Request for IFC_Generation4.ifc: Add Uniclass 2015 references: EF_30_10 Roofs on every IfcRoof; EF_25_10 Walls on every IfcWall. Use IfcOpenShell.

First a look at what the model holds.

```python
import ifcopenshell

model = ifcopenshell.open("IFC_Generation4.ifc")
print(model.schema)
print("classifications:", [c.Name for c in model.by_type("IfcClassification")])
for ifc_class in ("IfcDoor", "IfcRoof", "IfcStair", "IfcWall", "IfcWindow"):
    print(ifc_class, len(model.by_type(ifc_class)))
```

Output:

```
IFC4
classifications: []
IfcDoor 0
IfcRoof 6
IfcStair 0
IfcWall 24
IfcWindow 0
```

```python
import ifcopenshell
import ifcopenshell.api.classification

model = ifcopenshell.open("IFC_Generation4.ifc")

system = ifcopenshell.api.classification.add_classification(model, classification="Uniclass 2015")

codes = {
    "IfcRoof": ("EF_30_10", "Roofs"),
    "IfcWall": ("EF_25_10", "Walls"),
}
for ifc_class, (code, name) in codes.items():
    products = model.by_type(ifc_class)
    ifcopenshell.api.classification.add_reference(
        model, products=products, classification=system, identification=code, name=name
    )
    print(code, len(products))

model.write("IFC_Generation4_updated.ifc")
```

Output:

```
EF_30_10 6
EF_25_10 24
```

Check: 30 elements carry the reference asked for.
